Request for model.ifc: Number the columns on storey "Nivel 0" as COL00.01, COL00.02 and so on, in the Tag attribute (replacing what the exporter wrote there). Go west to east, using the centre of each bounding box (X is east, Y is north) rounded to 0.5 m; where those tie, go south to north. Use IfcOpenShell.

First a look at what the model holds.

```python
import ifcopenshell
import ifcopenshell.util.element
import ifcopenshell.util.placement

model = ifcopenshell.open("model.ifc")
print(model.schema)
storey = next(s for s in model.by_type("IfcBuildingStorey") if s.Name == "Nivel 0")
columns = [e for e in ifcopenshell.util.element.get_decomposition(storey) if e.is_a("IfcColumn")]
for e in sorted(columns, key=lambda e: e.id()):
    origin = ifcopenshell.util.placement.get_local_placement(e.ObjectPlacement)[:3, 3]
    print(e.id(), e.Tag, e.Name, origin.round(2) + 0.0, sep=" | ")
```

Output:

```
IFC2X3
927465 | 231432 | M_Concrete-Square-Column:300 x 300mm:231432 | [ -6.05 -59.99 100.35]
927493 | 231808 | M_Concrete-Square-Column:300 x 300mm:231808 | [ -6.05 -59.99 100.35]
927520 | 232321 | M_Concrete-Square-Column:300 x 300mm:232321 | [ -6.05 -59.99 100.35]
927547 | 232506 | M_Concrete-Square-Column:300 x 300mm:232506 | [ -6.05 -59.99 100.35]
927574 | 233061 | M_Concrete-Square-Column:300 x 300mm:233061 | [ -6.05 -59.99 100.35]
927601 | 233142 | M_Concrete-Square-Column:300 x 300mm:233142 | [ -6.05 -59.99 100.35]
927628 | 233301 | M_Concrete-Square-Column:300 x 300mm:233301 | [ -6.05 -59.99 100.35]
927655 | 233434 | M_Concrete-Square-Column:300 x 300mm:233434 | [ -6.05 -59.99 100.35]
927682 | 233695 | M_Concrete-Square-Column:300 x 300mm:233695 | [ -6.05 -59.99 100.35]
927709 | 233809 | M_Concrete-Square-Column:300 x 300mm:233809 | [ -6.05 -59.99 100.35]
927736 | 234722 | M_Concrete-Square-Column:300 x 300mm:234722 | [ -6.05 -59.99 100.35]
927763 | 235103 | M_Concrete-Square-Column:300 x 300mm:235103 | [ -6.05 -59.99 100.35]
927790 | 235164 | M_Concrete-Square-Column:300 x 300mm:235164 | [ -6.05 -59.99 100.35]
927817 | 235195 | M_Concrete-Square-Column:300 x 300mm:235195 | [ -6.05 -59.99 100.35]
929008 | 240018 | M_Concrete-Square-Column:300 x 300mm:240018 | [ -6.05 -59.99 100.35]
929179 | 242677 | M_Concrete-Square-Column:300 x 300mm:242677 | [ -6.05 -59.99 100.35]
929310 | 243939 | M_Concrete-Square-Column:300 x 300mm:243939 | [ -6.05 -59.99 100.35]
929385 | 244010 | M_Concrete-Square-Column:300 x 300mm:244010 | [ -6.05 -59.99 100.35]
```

```python
import ifcopenshell
import ifcopenshell.geom
import ifcopenshell.util.element
import ifcopenshell.util.shape

model = ifcopenshell.open("model.ifc")
settings = ifcopenshell.geom.settings()
settings.set("use-world-coords", True)


def centre(element):
    shape = ifcopenshell.geom.create_shape(settings, element)
    return ifcopenshell.util.shape.get_bbox_centroid(shape.geometry)


storey = next(s for s in model.by_type("IfcBuildingStorey") if s.Name == "Nivel 0")
columns = [e for e in ifcopenshell.util.element.get_decomposition(storey) if e.is_a("IfcColumn")]

# Insertion points can sit at a corner or the storey origin, so sort by the geometry (in metres).
centres = {e: centre(e) for e in columns}
columns.sort(key=lambda e: (round(centres[e][0] / 0.5), centres[e][1]))

for i, e in enumerate(columns, start=1):
    number = f"COL00.{i:02d}"
    e.Tag = number
    print(e.id(), number)

model.write("model_rev.ifc")
```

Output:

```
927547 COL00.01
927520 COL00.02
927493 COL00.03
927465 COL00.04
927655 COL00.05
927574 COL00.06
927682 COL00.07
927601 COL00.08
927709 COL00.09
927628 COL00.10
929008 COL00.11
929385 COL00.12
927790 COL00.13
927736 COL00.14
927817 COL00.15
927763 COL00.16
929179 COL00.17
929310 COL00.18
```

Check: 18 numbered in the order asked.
